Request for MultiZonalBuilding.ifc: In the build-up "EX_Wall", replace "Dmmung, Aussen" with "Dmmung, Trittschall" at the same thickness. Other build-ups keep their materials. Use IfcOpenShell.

First a look at what the model holds.

```python
import ifcopenshell
import ifcopenshell.util.element

model = ifcopenshell.open("MultiZonalBuilding.ifc")
print(model.schema)
for layer_set in model.by_type("IfcMaterialLayerSet"):
    if layer_set.LayerSetName == "EX_Wall":
        for layer in layer_set.MaterialLayers:
            print(layer.id(), layer.Material and layer.Material.Name, layer.LayerThickness, sep=" | ")
        print(len(ifcopenshell.util.element.get_elements_by_material(model, layer_set)), "elements and types use it")
print(sorted(m.Name for m in model.by_type("IfcMaterial") if m.Name)[:60])
```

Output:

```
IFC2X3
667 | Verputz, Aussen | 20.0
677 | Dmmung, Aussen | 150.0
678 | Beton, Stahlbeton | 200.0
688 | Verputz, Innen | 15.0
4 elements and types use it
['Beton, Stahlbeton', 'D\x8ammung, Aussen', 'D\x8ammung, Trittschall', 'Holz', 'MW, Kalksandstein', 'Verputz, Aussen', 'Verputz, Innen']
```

```python
import ifcopenshell
import ifcopenshell.api.material

model = ifcopenshell.open("MultiZonalBuilding.ifc")

layer_set = next(s for s in model.by_type("IfcMaterialLayerSet") if s.LayerSetName == "EX_Wall")
layer = next(l for l in layer_set.MaterialLayers if l.Material and l.Material.Name == 'D\x8ammung, Aussen')
material = next(m for m in model.by_type("IfcMaterial") if m.Name == 'D\x8ammung, Trittschall')

# Point this one layer at the other material; renaming the old one would change it everywhere.
ifcopenshell.api.material.edit_layer(model, layer=layer, attributes={}, material=material)

print([l.Material.Name if l.Material else None for l in layer_set.MaterialLayers])

model.write("MultiZonalBuilding-out.ifc")
```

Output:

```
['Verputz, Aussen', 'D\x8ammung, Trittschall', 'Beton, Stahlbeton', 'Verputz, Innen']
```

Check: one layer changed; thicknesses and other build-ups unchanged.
